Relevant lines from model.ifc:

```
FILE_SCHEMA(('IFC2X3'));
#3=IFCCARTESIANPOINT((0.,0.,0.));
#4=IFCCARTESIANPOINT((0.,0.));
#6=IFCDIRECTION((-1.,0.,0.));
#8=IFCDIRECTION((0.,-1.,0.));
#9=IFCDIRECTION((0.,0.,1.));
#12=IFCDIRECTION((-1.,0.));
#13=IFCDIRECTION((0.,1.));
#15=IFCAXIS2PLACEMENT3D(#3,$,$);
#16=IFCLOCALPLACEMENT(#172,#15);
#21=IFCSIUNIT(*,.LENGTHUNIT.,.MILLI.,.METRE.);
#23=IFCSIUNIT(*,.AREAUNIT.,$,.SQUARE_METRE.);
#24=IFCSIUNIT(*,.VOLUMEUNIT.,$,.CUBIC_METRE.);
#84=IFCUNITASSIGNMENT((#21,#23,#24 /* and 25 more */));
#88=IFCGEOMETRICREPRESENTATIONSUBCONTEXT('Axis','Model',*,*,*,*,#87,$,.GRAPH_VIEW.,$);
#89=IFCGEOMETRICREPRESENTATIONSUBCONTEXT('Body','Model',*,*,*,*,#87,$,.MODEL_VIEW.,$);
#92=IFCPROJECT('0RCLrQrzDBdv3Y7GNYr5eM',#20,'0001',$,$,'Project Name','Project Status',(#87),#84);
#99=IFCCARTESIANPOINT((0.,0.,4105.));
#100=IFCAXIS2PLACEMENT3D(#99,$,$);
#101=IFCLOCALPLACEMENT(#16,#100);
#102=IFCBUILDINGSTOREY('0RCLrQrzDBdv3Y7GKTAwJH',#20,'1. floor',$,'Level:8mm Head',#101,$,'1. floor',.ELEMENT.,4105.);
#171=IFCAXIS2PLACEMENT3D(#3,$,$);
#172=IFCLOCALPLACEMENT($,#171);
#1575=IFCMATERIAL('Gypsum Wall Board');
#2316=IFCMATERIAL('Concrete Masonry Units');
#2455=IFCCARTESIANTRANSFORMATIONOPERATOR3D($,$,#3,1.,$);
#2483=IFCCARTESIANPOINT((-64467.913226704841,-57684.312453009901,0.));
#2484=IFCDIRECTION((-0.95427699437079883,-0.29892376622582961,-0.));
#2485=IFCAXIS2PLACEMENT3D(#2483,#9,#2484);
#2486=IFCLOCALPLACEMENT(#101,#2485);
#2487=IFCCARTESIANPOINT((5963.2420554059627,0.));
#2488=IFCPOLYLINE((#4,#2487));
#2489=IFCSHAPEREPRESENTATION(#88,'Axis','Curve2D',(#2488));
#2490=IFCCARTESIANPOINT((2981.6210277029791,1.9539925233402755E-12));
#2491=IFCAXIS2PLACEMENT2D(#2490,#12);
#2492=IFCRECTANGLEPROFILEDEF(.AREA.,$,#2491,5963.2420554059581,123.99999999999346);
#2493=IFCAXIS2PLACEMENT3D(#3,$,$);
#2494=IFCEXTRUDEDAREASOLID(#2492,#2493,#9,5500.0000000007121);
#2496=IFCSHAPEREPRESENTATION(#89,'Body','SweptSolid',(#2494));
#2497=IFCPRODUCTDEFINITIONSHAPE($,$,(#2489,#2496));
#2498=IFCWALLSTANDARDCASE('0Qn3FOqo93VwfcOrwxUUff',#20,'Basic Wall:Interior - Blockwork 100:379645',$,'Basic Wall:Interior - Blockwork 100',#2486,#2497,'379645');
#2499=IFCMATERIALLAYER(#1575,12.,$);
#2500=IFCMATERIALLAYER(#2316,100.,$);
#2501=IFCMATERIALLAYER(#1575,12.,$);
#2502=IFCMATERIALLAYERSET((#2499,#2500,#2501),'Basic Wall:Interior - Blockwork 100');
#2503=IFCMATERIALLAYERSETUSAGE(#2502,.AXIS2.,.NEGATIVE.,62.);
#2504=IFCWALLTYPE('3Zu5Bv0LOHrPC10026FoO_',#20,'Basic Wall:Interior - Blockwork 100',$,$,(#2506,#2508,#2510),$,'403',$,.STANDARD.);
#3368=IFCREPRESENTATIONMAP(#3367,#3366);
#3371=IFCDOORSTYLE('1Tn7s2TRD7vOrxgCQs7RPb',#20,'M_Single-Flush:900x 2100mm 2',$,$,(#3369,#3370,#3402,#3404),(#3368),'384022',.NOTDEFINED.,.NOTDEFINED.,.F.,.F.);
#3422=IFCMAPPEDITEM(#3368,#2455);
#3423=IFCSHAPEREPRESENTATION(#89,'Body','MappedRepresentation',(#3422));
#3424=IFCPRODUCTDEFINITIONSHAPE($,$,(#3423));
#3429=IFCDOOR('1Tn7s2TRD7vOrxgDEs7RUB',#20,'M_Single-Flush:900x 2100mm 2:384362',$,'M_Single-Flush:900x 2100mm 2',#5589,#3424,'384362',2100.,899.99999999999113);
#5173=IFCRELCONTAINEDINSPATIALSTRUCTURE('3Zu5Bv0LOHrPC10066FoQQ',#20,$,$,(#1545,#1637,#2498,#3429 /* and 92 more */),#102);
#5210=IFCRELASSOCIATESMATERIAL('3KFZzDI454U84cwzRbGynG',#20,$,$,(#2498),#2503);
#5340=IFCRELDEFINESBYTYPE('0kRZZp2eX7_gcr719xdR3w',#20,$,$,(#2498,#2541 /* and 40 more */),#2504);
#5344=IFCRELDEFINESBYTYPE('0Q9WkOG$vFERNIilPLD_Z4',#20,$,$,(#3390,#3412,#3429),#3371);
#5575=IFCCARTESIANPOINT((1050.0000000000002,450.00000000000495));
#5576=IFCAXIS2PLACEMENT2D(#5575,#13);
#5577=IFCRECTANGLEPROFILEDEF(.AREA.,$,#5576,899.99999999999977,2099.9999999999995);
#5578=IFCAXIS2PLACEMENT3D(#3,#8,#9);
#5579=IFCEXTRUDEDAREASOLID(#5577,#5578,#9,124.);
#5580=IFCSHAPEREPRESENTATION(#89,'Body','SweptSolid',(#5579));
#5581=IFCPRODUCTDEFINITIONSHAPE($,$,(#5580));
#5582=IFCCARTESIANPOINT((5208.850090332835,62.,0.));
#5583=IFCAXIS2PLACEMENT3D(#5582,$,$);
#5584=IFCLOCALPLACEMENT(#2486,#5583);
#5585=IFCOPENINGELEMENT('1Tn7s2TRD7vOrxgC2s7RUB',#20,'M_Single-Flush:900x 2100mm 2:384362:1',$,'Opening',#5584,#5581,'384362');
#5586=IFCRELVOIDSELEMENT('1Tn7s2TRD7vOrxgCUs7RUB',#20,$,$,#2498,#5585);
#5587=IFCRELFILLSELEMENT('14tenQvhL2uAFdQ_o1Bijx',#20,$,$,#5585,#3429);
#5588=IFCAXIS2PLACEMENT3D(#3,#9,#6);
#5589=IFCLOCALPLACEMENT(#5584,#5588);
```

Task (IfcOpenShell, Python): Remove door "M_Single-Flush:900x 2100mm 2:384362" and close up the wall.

```python
import ifcopenshell
import ifcopenshell.api.feature
import ifcopenshell.api.root
import ifcopenshell.geom
import ifcopenshell.util.shape

model = ifcopenshell.open("model.ifc")
settings = ifcopenshell.geom.settings()


def volume(element):
    """Net volume in cubic metres, openings subtracted."""
    shape = ifcopenshell.geom.create_shape(settings, element)
    return ifcopenshell.util.shape.get_volume(shape.geometry)


door = model.by_guid("1Tn7s2TRD7vOrxgDEs7RUB")
opening = door.FillsVoids[0].RelatingOpeningElement
wall = opening.VoidsElements[0].RelatingBuildingElement
before = volume(wall)

ifcopenshell.api.root.remove_product(model, product=door)
ifcopenshell.api.feature.remove_feature(model, feature=opening)

after = volume(wall)

print(f"wall volume {before:.3f} -> {after:.3f} m3")

model.write("model-out.ifc")
```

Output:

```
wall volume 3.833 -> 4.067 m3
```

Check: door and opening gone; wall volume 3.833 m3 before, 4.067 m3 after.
